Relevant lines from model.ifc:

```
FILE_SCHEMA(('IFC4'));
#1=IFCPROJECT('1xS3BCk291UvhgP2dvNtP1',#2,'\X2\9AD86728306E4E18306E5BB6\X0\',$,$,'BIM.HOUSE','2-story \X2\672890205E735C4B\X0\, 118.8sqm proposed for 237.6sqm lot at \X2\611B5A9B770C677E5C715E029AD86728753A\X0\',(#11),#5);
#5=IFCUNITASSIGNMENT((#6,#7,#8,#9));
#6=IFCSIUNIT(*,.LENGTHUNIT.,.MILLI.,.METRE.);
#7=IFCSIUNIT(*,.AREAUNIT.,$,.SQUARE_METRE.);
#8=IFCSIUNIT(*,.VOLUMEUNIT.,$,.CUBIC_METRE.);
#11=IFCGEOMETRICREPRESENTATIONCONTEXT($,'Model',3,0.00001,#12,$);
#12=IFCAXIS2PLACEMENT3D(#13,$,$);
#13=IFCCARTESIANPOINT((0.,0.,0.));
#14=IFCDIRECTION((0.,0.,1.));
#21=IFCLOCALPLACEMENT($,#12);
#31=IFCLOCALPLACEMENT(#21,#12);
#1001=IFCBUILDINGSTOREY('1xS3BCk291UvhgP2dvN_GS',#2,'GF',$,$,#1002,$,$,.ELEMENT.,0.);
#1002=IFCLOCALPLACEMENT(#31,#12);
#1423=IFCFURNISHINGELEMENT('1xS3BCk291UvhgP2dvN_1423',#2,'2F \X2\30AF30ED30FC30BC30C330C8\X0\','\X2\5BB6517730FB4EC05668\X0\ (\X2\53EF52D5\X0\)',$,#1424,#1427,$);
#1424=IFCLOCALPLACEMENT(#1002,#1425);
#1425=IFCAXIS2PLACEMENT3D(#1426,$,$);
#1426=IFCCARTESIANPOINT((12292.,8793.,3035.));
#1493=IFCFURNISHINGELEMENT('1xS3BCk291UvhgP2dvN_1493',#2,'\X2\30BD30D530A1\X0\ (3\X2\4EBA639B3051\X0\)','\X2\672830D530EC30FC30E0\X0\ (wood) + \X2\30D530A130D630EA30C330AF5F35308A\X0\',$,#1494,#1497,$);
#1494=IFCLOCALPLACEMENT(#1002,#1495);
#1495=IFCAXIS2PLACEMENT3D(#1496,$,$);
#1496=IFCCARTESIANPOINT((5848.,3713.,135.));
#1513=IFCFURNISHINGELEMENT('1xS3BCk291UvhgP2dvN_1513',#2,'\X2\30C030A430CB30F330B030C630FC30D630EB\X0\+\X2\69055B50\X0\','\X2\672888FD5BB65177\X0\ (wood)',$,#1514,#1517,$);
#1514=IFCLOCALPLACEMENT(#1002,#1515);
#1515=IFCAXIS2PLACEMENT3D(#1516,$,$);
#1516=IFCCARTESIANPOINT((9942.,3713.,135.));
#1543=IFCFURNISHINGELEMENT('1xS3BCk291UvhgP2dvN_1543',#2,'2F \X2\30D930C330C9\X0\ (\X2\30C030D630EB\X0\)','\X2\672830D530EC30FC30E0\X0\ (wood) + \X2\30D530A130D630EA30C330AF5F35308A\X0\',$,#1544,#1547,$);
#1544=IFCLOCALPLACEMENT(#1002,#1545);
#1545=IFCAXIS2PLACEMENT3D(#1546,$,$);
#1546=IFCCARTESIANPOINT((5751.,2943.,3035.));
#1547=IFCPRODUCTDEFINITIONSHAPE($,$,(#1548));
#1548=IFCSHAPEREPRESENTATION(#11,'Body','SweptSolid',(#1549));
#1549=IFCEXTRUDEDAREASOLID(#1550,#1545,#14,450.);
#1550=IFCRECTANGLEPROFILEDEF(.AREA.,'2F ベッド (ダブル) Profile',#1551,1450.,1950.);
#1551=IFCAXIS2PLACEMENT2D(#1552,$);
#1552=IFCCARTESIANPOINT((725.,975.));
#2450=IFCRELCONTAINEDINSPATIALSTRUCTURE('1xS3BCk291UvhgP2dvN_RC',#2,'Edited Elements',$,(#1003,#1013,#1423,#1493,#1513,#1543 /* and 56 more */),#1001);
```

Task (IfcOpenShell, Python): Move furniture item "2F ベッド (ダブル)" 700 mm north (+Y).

```python
import ifcopenshell
import ifcopenshell.api.geometry
import ifcopenshell.util.placement
import ifcopenshell.util.unit

model = ifcopenshell.open("model.ifc")
unit_scale = ifcopenshell.util.unit.calculate_unit_scale(model)

item = model.by_id(1543)
matrix = ifcopenshell.util.placement.get_local_placement(item.ObjectPlacement)
matrix[1, 3] += 0.7 / unit_scale
ifcopenshell.api.geometry.edit_object_placement(model, product=item, matrix=matrix, is_si=False)

print(ifcopenshell.util.placement.get_local_placement(item.ObjectPlacement).round(3) + 0.0)

model.write("model_updated.ifc")
```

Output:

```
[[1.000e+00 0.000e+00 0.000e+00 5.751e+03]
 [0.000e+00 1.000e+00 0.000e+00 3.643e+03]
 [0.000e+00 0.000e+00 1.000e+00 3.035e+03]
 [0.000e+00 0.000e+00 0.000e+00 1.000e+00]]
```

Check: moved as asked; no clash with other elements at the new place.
